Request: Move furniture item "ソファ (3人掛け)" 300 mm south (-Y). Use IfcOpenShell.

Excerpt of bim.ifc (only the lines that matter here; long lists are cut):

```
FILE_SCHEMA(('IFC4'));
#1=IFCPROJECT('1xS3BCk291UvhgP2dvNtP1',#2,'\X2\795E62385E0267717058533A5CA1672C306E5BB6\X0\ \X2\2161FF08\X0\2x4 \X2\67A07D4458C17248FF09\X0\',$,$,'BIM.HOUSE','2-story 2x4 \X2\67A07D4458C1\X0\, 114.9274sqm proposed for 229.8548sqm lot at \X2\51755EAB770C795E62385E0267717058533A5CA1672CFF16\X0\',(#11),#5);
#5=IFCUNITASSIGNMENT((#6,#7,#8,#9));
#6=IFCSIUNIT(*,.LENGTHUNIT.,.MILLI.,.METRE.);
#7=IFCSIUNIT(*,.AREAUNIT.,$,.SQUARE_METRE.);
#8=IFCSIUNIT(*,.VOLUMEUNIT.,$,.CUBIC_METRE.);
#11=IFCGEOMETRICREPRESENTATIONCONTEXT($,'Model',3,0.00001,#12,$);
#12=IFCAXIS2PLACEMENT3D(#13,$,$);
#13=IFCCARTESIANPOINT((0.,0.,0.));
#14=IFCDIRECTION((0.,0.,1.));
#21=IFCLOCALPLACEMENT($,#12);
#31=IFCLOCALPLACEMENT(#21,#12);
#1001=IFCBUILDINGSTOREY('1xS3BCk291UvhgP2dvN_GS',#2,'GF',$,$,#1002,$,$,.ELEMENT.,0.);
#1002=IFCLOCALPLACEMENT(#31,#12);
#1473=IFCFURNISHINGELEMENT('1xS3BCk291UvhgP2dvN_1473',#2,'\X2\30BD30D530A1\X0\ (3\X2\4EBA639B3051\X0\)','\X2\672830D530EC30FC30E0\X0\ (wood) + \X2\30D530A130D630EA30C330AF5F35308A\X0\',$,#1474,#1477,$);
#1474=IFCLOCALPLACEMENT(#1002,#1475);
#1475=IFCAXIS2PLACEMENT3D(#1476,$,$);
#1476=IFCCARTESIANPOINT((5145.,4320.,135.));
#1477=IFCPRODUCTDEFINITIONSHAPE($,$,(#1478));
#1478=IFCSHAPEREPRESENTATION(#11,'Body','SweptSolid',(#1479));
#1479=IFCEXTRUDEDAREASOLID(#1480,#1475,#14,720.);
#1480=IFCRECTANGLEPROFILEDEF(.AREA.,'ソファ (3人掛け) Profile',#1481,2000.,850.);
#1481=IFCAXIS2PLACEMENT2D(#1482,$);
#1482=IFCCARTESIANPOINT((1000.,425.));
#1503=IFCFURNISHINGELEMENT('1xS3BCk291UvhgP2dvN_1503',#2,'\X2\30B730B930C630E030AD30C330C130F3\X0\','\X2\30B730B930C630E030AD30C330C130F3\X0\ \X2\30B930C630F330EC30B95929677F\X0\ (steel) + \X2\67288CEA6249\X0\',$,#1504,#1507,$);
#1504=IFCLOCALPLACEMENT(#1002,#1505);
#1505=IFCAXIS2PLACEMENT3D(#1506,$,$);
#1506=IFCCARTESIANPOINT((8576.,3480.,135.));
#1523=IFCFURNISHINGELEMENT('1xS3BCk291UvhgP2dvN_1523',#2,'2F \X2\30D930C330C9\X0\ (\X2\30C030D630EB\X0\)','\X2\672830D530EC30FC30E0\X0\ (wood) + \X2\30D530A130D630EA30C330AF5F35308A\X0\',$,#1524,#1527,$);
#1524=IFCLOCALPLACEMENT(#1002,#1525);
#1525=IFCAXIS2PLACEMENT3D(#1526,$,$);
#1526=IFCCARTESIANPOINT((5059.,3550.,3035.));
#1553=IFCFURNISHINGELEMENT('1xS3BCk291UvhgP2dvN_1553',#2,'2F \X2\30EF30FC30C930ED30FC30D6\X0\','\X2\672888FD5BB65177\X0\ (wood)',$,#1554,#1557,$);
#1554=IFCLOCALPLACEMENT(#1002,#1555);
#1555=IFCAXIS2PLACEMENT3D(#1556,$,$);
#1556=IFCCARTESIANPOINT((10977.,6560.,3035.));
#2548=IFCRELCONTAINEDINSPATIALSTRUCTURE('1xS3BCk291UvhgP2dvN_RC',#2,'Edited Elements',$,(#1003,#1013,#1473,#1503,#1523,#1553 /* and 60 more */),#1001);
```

```python
import ifcopenshell
import ifcopenshell.api.geometry
import ifcopenshell.util.placement
import ifcopenshell.util.unit

model = ifcopenshell.open("bim.ifc")
unit_scale = ifcopenshell.util.unit.calculate_unit_scale(model)

item = model.by_id(1473)
matrix = ifcopenshell.util.placement.get_local_placement(item.ObjectPlacement)
matrix[1, 3] -= 0.3 / unit_scale
ifcopenshell.api.geometry.edit_object_placement(model, product=item, matrix=matrix, is_si=False)

print(ifcopenshell.util.placement.get_local_placement(item.ObjectPlacement).round(3) + 0.0)

model.write("bim_v2.ifc")
```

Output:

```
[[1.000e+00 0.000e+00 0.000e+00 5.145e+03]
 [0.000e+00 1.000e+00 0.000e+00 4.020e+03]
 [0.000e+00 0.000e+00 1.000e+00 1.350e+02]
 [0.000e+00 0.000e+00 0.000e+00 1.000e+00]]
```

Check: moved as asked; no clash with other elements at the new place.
